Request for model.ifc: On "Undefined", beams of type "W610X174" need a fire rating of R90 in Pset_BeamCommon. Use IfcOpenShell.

First a look at what the model holds.

```python
import ifcopenshell
import ifcopenshell.util.element

model = ifcopenshell.open("model.ifc")
print(model.schema)
storey = next(s for s in model.by_type("IfcBuildingStorey") if s.Name == "Undefined")
beams = [e for e in ifcopenshell.util.element.get_decomposition(storey) if e.is_a("IfcBeam")]
seen = {}
for e in beams:
    element_type = ifcopenshell.util.element.get_type(e)
    key = (element_type.Name if element_type != e and element_type else None, ifcopenshell.util.element.get_pset(e, "Pset_BeamCommon", "FireRating"))
    seen[key] = seen.get(key, 0) + 1
for (name, value), count in sorted(seen.items(), key=str):
    print(count, "x", name, "|", value)
```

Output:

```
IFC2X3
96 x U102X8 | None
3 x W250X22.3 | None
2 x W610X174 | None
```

```python
import ifcopenshell
import ifcopenshell.api.pset
import ifcopenshell.util.element

model = ifcopenshell.open("model.ifc")

storey = next(s for s in model.by_type("IfcBuildingStorey") if s.Name == "Undefined")
beams = [e for e in ifcopenshell.util.element.get_decomposition(storey) if e.is_a("IfcBeam")]

count = 0
for e in beams:
    element_type = ifcopenshell.util.element.get_type(e)
    if element_type in (None, e) or element_type.Name != "W610X174":
        continue
    found = ifcopenshell.util.element.get_pset(e, "Pset_BeamCommon", should_inherit=False)
    if found:
        pset = model.by_id(found["id"])
        if len(ifcopenshell.util.element.get_elements_by_pset(pset)) > 1:
            pset = ifcopenshell.api.pset.unshare_pset(model, products=[e], pset=pset)[0]
    else:
        pset = ifcopenshell.api.pset.add_pset(model, product=e, name="Pset_BeamCommon")
    ifcopenshell.api.pset.edit_pset(model, pset=pset, properties={"FireRating": "R90"})
    count += 1

print(count, "beams updated")

model.write("model_edited.ifc")
```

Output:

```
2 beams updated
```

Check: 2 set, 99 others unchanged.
